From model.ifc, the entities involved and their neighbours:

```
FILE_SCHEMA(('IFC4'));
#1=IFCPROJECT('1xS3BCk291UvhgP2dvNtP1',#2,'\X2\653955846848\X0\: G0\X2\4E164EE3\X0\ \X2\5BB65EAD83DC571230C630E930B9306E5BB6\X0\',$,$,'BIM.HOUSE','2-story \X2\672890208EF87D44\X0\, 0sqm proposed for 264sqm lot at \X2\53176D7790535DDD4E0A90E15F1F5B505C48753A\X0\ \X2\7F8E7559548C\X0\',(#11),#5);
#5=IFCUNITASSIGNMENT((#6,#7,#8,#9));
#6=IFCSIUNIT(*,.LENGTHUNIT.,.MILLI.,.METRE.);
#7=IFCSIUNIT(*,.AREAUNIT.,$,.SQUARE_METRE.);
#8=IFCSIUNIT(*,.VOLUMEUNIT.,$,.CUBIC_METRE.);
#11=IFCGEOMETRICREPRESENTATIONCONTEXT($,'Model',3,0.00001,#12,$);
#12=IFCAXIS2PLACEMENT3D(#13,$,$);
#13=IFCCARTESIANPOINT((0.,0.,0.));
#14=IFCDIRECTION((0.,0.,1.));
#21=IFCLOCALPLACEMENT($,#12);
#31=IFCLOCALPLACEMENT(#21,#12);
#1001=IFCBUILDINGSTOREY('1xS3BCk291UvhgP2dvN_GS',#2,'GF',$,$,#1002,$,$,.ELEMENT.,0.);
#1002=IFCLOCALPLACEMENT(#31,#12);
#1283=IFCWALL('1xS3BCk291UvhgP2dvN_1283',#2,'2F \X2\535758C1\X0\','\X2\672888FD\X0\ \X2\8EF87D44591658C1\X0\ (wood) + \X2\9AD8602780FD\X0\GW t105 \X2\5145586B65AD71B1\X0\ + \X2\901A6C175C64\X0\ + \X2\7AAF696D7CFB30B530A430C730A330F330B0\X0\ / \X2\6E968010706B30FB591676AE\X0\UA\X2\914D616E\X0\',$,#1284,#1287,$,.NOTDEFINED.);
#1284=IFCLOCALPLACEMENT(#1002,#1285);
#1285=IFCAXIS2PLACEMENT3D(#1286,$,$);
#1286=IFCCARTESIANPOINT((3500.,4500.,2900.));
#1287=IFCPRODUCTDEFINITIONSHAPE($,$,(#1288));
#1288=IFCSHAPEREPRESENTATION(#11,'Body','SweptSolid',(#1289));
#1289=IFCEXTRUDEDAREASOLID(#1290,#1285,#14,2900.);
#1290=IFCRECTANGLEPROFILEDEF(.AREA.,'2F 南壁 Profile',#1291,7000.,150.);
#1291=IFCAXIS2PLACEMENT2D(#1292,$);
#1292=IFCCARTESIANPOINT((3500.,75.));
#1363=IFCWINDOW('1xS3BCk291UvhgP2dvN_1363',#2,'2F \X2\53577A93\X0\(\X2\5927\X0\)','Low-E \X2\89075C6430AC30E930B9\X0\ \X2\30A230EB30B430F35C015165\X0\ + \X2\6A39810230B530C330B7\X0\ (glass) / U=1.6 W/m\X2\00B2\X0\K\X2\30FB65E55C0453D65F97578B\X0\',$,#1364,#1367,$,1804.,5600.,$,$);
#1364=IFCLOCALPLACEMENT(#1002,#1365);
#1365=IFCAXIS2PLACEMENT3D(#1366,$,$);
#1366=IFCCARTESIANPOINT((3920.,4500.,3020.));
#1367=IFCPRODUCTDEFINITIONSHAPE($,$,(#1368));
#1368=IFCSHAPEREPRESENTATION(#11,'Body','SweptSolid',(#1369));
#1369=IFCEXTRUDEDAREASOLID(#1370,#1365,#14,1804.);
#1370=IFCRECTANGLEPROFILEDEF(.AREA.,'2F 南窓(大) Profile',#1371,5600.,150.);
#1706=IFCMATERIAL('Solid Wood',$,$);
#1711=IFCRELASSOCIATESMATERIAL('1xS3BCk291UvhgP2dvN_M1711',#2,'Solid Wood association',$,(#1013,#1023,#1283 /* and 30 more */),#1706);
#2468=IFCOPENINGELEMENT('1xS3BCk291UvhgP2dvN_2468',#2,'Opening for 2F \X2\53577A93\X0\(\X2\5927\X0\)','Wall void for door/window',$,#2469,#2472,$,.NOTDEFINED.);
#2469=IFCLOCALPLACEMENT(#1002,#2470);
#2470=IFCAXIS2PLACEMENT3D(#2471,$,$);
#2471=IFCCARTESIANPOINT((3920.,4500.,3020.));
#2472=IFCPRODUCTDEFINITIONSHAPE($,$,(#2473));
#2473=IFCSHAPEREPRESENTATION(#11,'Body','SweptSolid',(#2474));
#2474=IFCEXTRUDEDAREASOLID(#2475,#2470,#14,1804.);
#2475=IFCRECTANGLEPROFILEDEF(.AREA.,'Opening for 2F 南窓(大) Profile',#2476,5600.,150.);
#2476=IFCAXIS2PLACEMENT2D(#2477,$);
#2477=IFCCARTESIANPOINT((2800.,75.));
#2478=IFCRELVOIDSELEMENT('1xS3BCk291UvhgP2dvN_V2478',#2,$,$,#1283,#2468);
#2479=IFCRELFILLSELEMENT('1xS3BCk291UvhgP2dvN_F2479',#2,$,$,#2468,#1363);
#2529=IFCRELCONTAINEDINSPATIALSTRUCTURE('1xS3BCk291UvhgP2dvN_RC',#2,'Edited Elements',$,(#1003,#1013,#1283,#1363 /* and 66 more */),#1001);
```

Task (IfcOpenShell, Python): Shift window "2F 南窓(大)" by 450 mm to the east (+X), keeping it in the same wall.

```python
import ifcopenshell
import ifcopenshell.api.geometry
import ifcopenshell.util.placement

model = ifcopenshell.open("model.ifc")

window = model.by_guid("1xS3BCk291UvhgP2dvN_1363")
opening = window.FillsVoids[0].RelatingOpeningElement
wall = opening.VoidsElements[0].RelatingBuildingElement

wall_matrix = ifcopenshell.util.placement.get_local_placement(wall.ObjectPlacement)
shift = wall_matrix[:3, 0] * 450.0
before = ifcopenshell.util.placement.get_local_placement(window.ObjectPlacement)[:3, 3].copy()

# The window is not placed relative to its opening, so move both.
for product in (opening, window):
    matrix = ifcopenshell.util.placement.get_local_placement(product.ObjectPlacement)
    matrix[:3, 3] += shift
    ifcopenshell.api.geometry.edit_object_placement(model, product=product, matrix=matrix, is_si=False)

after = ifcopenshell.util.placement.get_local_placement(window.ObjectPlacement)[:3, 3]
print("window moved by", (after - before).round(3) + 0.0)

model.write("model-out.ifc")
```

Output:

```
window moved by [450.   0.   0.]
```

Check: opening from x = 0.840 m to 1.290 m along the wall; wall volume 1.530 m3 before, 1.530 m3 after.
